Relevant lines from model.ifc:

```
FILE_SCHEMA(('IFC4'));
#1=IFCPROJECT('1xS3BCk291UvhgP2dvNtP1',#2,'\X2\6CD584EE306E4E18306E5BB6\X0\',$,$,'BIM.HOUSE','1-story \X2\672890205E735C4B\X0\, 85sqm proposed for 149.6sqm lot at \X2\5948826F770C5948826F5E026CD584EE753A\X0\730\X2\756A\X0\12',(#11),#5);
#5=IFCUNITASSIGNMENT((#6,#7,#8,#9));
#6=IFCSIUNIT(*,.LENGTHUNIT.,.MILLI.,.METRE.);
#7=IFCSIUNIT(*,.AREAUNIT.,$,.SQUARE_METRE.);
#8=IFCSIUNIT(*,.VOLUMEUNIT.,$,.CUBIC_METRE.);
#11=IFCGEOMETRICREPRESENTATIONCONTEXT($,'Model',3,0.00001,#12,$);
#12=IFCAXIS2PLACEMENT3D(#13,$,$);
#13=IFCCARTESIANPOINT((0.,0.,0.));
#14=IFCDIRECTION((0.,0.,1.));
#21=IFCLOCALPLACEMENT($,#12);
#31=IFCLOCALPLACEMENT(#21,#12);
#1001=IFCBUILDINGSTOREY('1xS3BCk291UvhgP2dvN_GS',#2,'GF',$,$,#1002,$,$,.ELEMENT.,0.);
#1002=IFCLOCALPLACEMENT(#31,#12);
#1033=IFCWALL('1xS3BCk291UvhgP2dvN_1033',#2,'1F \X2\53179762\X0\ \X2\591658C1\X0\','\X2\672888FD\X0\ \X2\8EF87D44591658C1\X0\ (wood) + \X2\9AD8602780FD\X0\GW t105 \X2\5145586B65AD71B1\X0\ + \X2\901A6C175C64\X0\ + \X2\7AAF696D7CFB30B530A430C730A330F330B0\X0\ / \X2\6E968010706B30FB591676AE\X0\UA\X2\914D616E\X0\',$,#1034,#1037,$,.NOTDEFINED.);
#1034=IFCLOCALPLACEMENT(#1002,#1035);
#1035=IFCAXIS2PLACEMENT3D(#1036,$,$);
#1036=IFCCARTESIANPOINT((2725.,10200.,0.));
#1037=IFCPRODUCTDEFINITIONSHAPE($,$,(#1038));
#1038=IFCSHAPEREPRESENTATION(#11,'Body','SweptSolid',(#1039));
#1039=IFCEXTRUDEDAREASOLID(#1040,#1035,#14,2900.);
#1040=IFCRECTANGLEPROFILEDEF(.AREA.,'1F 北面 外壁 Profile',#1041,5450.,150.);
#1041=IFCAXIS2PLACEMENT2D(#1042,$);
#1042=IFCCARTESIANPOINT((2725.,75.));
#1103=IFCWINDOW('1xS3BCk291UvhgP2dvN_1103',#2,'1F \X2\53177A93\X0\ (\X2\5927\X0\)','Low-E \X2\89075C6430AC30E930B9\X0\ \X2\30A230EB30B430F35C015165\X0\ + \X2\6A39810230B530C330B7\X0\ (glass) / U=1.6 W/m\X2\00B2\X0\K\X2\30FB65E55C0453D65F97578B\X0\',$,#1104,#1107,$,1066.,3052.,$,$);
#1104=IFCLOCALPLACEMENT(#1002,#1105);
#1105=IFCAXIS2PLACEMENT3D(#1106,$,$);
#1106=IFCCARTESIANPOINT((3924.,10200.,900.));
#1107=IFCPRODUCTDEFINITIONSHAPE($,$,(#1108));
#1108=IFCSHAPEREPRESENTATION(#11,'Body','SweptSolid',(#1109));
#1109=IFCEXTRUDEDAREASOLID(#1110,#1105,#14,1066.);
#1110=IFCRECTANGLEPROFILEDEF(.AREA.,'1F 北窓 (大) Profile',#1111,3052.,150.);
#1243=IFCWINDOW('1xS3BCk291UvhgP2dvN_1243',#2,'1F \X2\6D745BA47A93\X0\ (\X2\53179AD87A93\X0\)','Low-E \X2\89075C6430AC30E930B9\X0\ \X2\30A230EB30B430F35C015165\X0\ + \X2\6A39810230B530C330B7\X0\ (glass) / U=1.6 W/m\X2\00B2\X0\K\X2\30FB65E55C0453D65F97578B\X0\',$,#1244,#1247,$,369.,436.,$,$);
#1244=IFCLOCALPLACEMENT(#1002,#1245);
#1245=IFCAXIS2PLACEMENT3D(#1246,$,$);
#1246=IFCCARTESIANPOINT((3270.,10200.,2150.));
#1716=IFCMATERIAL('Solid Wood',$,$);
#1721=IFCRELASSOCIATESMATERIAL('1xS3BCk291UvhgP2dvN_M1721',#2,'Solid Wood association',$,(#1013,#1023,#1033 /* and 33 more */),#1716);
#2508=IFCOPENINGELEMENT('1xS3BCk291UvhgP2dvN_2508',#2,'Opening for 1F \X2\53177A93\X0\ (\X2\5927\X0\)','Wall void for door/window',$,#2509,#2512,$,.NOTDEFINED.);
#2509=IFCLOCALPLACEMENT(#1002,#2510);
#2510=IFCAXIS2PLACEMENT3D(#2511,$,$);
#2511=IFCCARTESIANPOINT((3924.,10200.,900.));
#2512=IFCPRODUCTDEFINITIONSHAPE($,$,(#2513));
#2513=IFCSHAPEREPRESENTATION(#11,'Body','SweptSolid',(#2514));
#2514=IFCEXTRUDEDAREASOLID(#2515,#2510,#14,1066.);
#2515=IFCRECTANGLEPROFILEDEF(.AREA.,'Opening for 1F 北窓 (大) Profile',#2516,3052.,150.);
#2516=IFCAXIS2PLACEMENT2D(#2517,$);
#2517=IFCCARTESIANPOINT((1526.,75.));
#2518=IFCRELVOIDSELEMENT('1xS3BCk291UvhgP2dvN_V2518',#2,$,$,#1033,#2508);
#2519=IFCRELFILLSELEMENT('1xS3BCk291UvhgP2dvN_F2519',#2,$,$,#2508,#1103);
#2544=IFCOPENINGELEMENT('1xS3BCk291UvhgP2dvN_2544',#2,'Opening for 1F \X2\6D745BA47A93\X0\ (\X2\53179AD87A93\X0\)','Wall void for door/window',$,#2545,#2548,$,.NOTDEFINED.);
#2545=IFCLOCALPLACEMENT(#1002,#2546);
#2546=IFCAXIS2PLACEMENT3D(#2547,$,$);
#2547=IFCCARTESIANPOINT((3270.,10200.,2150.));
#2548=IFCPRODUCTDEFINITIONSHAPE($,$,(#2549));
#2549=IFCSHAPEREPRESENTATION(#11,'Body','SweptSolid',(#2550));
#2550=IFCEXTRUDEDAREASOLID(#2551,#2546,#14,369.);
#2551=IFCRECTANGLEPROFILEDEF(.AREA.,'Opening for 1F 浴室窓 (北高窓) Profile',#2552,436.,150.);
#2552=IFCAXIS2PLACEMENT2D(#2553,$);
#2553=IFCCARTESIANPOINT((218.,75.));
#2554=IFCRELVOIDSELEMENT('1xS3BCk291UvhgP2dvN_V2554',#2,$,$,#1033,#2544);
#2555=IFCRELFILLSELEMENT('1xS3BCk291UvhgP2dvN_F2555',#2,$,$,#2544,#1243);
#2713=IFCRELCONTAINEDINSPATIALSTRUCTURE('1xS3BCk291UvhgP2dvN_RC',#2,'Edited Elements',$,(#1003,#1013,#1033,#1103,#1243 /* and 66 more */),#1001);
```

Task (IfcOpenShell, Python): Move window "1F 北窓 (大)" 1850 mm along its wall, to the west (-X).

```python
import ifcopenshell
import ifcopenshell.api.geometry
import ifcopenshell.util.placement
import ifcopenshell.util.unit

model = ifcopenshell.open("model.ifc")
unit_scale = ifcopenshell.util.unit.calculate_unit_scale(model)

window = model.by_guid("1xS3BCk291UvhgP2dvN_1103")
opening = window.FillsVoids[0].RelatingOpeningElement
wall = opening.VoidsElements[0].RelatingBuildingElement

wall_matrix = ifcopenshell.util.placement.get_local_placement(wall.ObjectPlacement)
shift = wall_matrix[:3, 0] * -1.85 / unit_scale
before = ifcopenshell.util.placement.get_local_placement(window.ObjectPlacement)[:3, 3].copy()

# The window is not placed relative to its opening, so move both.
for product in (opening, window):
    matrix = ifcopenshell.util.placement.get_local_placement(product.ObjectPlacement)
    matrix[:3, 3] += shift
    ifcopenshell.api.geometry.edit_object_placement(model, product=product, matrix=matrix, is_si=False)

after = ifcopenshell.util.placement.get_local_placement(window.ObjectPlacement)[:3, 3]
print("window moved by", (after - before).round(3) + 0.0)

model.write("model_rev.ifc")
```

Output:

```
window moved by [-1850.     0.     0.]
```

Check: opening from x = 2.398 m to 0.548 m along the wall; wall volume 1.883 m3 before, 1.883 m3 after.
